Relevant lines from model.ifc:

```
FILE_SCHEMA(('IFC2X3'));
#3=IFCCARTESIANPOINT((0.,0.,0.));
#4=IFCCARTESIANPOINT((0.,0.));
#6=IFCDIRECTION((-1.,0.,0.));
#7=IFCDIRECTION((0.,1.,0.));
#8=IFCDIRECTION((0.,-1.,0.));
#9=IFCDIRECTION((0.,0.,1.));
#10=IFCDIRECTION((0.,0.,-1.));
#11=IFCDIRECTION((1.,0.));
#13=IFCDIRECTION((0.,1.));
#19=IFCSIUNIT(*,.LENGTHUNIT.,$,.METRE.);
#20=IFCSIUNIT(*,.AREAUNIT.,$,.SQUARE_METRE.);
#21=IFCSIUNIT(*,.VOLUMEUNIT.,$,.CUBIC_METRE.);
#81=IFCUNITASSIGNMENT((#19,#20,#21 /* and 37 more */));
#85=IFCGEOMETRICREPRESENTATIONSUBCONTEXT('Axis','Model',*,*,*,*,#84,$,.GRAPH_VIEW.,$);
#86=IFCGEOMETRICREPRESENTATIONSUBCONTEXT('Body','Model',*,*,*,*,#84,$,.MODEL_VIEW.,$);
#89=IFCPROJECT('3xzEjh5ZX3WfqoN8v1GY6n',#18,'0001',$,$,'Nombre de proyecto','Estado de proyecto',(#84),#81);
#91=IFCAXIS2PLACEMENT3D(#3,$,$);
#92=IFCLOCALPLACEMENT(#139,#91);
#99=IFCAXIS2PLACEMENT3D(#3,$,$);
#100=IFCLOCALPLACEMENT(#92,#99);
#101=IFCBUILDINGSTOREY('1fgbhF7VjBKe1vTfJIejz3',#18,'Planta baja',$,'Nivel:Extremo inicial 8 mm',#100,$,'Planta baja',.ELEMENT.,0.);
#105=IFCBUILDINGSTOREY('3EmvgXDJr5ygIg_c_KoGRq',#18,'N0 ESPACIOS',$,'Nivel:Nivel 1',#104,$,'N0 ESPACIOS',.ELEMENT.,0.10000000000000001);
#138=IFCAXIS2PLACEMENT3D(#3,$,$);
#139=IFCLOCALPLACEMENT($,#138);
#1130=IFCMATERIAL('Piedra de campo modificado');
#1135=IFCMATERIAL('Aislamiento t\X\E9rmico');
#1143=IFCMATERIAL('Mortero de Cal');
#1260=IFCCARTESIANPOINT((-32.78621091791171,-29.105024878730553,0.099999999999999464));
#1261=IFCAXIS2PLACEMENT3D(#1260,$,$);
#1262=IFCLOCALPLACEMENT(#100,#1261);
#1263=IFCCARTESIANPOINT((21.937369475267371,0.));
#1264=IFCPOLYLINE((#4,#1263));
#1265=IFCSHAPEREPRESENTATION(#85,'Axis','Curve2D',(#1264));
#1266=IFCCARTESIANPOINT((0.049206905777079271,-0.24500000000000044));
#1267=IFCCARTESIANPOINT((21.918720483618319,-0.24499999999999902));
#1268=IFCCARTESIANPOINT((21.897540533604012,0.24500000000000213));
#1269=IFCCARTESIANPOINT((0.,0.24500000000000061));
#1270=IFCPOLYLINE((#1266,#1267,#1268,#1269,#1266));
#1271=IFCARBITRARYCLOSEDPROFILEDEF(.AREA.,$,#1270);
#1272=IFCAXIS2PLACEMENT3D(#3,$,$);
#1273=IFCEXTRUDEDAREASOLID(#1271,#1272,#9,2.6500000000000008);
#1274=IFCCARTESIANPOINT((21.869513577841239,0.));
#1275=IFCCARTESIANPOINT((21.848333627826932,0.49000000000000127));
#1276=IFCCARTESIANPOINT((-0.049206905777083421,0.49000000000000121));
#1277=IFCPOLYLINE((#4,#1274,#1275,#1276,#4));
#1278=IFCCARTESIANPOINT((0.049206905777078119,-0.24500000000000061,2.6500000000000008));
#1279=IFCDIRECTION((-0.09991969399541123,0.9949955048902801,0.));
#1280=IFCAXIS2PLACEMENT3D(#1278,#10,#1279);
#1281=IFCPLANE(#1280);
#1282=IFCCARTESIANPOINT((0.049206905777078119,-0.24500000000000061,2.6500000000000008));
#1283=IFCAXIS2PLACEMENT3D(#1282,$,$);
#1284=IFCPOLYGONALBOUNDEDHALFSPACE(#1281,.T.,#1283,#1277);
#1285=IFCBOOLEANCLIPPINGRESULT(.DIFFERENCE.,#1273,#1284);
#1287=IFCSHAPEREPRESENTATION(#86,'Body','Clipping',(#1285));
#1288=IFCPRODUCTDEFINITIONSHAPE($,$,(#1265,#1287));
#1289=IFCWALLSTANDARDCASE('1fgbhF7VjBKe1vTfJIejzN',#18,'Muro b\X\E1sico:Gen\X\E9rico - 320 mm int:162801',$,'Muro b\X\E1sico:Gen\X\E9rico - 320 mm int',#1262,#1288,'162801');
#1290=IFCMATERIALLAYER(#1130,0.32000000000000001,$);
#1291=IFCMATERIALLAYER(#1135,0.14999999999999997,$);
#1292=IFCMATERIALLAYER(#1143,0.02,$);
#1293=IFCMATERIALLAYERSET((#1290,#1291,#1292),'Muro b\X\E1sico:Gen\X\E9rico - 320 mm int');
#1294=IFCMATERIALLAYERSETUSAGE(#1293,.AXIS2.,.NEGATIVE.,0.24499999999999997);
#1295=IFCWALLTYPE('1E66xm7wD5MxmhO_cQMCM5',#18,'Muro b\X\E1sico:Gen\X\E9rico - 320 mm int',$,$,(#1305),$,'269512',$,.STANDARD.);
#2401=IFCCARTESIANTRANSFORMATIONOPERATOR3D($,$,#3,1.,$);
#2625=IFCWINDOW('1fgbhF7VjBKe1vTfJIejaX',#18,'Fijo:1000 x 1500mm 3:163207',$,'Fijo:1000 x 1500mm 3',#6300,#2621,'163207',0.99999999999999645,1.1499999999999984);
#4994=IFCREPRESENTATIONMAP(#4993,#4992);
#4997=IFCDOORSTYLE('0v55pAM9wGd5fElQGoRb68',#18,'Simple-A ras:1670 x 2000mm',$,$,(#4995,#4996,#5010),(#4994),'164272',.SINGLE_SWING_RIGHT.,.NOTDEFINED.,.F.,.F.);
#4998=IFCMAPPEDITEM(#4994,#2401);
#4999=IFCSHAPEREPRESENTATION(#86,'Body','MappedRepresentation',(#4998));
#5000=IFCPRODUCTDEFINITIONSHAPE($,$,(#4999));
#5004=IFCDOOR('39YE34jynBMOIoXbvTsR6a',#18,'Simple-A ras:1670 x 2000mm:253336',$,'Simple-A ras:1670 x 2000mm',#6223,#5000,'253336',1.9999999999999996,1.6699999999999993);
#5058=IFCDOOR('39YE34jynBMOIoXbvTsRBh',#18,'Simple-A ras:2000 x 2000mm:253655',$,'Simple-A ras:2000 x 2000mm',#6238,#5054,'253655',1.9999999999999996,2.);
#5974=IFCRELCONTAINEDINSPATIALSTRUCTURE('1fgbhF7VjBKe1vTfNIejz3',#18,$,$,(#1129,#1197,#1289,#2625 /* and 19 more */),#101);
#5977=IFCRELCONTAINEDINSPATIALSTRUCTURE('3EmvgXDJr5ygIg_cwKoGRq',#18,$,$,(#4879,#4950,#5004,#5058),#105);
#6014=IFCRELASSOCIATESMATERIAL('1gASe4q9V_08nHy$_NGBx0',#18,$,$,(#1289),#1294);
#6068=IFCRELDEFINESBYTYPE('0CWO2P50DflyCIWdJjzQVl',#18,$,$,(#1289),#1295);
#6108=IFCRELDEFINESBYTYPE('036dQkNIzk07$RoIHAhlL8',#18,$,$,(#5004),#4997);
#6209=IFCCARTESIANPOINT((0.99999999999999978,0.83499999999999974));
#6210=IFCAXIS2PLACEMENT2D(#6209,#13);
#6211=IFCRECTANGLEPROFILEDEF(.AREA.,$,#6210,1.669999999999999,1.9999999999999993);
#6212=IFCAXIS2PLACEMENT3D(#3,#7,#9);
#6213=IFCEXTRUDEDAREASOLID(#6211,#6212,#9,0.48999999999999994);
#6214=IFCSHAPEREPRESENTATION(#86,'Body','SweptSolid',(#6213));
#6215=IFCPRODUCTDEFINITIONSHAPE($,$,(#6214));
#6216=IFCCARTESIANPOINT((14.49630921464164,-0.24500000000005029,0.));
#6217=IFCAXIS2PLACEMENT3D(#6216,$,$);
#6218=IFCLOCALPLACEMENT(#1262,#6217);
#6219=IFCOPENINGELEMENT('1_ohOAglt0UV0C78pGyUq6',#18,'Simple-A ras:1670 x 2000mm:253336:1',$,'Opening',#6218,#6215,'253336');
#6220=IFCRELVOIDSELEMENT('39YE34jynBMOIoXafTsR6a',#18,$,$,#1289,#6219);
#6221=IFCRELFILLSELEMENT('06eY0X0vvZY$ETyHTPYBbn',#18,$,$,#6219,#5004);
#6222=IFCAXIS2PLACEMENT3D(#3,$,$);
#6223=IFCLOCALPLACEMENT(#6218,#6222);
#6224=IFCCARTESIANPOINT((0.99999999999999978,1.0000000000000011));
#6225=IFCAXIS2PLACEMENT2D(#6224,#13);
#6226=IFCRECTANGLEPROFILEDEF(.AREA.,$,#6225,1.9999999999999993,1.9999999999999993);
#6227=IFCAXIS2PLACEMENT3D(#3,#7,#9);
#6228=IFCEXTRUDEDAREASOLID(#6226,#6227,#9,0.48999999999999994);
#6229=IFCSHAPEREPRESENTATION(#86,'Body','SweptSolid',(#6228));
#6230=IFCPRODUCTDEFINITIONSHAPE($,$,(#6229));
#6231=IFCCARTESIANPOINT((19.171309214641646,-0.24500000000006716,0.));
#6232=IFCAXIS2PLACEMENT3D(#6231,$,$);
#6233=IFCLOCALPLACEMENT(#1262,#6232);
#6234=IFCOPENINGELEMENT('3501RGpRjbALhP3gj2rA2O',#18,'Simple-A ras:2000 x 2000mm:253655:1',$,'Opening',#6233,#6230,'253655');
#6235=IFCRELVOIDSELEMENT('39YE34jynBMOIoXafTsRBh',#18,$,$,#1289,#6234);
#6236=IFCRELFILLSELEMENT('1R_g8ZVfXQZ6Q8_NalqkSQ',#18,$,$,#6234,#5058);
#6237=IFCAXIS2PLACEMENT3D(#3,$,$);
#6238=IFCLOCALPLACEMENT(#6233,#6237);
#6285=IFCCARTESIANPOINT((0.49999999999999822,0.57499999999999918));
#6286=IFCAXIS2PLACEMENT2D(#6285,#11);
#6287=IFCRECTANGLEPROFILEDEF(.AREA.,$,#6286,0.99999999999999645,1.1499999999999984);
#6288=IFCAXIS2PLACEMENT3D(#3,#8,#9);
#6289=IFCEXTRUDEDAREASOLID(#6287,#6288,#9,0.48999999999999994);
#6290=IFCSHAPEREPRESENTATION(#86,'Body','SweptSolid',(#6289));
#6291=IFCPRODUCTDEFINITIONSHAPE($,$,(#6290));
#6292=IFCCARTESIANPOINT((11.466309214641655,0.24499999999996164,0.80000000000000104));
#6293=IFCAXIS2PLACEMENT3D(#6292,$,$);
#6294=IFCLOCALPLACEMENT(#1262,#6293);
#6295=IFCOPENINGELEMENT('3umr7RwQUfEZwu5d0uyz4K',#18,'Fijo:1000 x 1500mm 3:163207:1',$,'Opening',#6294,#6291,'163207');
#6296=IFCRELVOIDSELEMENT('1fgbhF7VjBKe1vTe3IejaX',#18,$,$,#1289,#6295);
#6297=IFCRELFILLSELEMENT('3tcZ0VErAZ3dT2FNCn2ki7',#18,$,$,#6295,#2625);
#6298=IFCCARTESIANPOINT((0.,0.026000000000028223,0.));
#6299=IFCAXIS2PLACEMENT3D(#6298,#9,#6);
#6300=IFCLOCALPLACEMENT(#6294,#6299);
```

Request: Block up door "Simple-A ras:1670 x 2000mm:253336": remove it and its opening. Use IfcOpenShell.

```python
import ifcopenshell
import ifcopenshell.api.feature
import ifcopenshell.api.root
import ifcopenshell.geom
import ifcopenshell.util.shape

model = ifcopenshell.open("model.ifc")
settings = ifcopenshell.geom.settings()


def volume(element):
    """Net volume in cubic metres, openings subtracted."""
    shape = ifcopenshell.geom.create_shape(settings, element)
    return ifcopenshell.util.shape.get_volume(shape.geometry)


door = model.by_guid("39YE34jynBMOIoXbvTsR6a")
opening = door.FillsVoids[0].RelatingOpeningElement
wall = opening.VoidsElements[0].RelatingBuildingElement
before = volume(wall)

ifcopenshell.api.root.remove_product(model, product=door)
ifcopenshell.api.feature.remove_feature(model, feature=opening)

after = volume(wall)

print(f"wall volume {before:.3f} -> {after:.3f} m3")

model.write("model_updated.ifc")
```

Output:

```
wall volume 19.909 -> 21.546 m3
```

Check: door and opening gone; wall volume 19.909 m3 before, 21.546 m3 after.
